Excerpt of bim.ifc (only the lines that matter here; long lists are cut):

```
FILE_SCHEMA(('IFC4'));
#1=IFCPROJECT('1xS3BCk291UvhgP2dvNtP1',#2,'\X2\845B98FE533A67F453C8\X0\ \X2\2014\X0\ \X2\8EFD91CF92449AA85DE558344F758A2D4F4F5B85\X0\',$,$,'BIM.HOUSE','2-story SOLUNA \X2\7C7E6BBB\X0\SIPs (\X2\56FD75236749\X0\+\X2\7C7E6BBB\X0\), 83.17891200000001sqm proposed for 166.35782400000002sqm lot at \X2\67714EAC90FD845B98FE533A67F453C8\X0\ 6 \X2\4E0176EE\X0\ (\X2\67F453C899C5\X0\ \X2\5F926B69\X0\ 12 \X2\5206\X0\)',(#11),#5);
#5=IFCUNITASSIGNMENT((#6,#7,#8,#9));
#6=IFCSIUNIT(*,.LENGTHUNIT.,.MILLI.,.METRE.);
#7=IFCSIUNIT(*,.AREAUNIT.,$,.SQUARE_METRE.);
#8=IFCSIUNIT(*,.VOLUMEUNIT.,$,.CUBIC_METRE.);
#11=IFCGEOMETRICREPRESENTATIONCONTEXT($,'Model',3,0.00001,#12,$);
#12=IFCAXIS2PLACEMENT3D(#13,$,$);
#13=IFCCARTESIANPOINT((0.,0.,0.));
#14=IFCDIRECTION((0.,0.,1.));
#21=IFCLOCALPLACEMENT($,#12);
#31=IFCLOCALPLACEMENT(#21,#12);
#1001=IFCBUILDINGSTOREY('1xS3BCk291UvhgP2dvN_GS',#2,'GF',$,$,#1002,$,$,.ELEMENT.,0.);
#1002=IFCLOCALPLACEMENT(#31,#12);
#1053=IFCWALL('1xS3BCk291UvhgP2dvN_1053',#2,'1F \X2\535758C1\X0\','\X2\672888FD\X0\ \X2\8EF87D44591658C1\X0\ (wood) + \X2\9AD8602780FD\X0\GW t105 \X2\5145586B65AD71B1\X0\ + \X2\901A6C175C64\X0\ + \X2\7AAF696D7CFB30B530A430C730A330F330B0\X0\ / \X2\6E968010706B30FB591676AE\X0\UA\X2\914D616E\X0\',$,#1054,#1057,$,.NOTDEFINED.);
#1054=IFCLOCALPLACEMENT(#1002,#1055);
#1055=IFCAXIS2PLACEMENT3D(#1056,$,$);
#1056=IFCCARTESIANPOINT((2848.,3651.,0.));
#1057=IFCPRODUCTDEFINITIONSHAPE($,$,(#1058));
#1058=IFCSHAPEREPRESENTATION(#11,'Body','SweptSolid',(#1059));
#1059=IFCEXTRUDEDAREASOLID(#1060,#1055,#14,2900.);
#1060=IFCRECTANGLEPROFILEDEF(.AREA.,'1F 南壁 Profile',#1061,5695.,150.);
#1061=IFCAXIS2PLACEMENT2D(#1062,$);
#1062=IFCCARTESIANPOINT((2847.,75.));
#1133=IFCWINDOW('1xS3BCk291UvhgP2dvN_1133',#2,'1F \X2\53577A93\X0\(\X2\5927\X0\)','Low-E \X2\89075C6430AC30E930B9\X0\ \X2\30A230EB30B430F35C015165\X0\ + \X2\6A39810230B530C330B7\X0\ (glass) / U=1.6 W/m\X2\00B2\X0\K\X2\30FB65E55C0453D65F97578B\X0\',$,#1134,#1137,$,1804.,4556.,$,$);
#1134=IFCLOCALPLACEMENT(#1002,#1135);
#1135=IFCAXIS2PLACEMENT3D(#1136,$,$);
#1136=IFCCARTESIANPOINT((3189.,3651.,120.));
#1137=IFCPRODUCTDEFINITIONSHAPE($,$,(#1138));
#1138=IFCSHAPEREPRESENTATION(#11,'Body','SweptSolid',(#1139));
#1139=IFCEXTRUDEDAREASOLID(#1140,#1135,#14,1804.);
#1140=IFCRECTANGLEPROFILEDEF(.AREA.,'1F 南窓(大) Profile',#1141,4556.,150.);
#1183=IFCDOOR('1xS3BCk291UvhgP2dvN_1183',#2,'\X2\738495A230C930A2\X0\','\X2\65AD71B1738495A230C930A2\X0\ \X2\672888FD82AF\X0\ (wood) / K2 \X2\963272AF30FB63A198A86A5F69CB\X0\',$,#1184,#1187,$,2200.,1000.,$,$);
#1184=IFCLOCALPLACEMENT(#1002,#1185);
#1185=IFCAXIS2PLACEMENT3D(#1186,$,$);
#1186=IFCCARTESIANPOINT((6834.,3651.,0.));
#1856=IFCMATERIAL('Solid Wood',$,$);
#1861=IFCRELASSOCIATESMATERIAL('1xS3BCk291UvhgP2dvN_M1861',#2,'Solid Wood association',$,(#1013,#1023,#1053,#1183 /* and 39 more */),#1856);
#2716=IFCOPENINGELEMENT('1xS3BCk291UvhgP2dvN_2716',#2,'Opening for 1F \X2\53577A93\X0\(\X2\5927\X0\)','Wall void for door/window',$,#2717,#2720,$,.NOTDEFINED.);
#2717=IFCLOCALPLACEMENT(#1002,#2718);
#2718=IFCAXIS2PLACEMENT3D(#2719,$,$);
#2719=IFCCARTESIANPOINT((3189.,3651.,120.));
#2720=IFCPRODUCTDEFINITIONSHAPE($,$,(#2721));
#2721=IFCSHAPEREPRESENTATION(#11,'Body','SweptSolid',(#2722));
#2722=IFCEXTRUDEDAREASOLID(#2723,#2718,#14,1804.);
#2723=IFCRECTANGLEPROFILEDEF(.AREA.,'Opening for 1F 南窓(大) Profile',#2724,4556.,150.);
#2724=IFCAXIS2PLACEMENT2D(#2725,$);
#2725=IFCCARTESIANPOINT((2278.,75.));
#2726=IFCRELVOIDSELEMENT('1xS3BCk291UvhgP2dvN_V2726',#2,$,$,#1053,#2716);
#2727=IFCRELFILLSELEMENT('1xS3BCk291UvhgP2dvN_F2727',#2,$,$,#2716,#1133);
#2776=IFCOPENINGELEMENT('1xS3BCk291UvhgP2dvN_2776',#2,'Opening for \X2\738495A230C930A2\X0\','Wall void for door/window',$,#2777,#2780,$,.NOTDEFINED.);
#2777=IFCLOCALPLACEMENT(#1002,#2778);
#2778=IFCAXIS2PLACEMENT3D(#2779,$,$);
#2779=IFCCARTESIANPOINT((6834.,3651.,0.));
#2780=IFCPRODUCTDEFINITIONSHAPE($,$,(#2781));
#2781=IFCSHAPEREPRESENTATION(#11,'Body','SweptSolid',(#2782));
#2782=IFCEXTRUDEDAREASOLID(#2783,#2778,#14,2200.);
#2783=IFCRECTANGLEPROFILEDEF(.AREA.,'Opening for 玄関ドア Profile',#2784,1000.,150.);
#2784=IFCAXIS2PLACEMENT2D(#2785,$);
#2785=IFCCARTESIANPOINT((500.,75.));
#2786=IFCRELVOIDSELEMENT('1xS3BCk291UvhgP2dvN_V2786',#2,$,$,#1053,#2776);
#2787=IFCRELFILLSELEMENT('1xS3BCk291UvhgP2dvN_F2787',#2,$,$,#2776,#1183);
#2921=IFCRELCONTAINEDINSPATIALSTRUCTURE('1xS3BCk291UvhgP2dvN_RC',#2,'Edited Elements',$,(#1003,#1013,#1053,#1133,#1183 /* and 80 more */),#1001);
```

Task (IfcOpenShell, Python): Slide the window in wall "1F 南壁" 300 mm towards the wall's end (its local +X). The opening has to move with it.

```python
import ifcopenshell
import ifcopenshell.api.geometry
import ifcopenshell.util.placement

model = ifcopenshell.open("bim.ifc")

window = model.by_id(1133)
opening = window.FillsVoids[0].RelatingOpeningElement
wall = opening.VoidsElements[0].RelatingBuildingElement

wall_matrix = ifcopenshell.util.placement.get_local_placement(wall.ObjectPlacement)
shift = wall_matrix[:3, 0] * 300.0
before = ifcopenshell.util.placement.get_local_placement(window.ObjectPlacement)[:3, 3].copy()

# The window is not placed relative to its opening, so move both.
for product in (opening, window):
    matrix = ifcopenshell.util.placement.get_local_placement(product.ObjectPlacement)
    matrix[:3, 3] += shift
    ifcopenshell.api.geometry.edit_object_placement(model, product=product, matrix=matrix, is_si=False)

after = ifcopenshell.util.placement.get_local_placement(window.ObjectPlacement)[:3, 3]
print("window moved by", (after - before).round(3) + 0.0)

model.write("bim-out.ifc")
```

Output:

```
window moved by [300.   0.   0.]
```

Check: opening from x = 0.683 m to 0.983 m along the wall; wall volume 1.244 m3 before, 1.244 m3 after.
